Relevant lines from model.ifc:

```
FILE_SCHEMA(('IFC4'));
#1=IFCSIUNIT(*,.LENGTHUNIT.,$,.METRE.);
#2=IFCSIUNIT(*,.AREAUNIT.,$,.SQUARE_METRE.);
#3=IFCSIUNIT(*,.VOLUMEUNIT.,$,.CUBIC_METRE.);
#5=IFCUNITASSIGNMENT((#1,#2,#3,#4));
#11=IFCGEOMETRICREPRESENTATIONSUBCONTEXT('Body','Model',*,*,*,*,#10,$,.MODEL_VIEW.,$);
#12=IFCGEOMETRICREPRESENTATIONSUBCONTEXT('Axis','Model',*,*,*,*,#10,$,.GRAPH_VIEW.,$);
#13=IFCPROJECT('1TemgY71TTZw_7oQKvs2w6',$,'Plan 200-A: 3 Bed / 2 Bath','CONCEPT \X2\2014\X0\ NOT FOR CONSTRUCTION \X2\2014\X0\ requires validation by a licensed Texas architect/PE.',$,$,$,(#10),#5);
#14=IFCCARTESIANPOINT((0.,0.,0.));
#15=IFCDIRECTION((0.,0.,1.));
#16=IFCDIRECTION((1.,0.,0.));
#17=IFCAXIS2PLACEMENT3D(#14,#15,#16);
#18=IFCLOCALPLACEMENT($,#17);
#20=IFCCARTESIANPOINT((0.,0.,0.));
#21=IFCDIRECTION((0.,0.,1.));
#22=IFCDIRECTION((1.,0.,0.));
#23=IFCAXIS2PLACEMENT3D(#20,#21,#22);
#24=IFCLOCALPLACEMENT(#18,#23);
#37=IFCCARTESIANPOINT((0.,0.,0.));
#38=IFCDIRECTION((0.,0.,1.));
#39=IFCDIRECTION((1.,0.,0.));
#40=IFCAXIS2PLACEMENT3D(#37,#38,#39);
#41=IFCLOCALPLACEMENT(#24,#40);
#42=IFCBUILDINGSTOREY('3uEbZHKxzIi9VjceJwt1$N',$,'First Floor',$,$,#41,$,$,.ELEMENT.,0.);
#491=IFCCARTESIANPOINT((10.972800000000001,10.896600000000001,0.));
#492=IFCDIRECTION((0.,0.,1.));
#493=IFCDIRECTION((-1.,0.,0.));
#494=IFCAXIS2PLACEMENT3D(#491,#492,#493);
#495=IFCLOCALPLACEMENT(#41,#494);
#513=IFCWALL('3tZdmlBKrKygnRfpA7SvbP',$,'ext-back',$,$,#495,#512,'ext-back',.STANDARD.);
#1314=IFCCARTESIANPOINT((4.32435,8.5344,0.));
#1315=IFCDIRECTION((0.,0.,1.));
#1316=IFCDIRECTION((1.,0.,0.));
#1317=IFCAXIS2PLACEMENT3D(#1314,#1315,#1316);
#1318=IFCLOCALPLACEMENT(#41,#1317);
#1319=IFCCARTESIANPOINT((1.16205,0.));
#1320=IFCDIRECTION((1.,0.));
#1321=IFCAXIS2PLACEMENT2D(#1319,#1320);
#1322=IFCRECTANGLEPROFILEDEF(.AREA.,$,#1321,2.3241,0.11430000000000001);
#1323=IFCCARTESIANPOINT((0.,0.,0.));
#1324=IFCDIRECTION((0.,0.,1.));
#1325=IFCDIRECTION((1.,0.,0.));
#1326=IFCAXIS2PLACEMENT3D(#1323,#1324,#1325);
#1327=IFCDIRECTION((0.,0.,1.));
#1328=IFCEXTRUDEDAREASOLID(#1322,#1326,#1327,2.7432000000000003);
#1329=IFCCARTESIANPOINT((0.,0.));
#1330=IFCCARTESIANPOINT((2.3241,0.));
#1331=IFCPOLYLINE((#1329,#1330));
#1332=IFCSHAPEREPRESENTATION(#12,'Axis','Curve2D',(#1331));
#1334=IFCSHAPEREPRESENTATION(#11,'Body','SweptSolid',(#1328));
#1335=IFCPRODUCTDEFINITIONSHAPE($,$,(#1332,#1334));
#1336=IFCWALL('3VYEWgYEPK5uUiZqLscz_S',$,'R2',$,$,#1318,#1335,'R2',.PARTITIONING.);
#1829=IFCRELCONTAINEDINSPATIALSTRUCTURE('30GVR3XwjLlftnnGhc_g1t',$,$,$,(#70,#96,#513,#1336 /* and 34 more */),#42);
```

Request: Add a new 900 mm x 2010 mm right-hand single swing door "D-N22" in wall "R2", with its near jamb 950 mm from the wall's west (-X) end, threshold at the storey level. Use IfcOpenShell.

```python
import numpy as np
import ifcopenshell
import ifcopenshell.api.feature
import ifcopenshell.api.geometry
import ifcopenshell.api.root
import ifcopenshell.api.spatial
import ifcopenshell.geom
import ifcopenshell.util.element
import ifcopenshell.util.placement
import ifcopenshell.util.representation
import ifcopenshell.util.shape
import ifcopenshell.util.unit

model = ifcopenshell.open("model.ifc")
unit_scale = ifcopenshell.util.unit.calculate_unit_scale(model)
settings = ifcopenshell.geom.settings()


def volume(element):
    """Net volume in cubic metres, openings subtracted."""
    shape = ifcopenshell.geom.create_shape(settings, element)
    return ifcopenshell.util.shape.get_volume(shape.geometry)


wall = model.by_guid("3VYEWgYEPK5uUiZqLscz_S")
storey = ifcopenshell.util.element.get_container(wall, ifc_class="IfcBuildingStorey")
context = ifcopenshell.util.representation.get_context(model, "Model", "Body", "MODEL_VIEW")
before = volume(wall)

width, height, from_end, sill = 0.9, 2.01, 0.95, 0.0  # metres

# The wall runs along its own X axis, and the end named is its -X end.
wall_shape = ifcopenshell.geom.create_shape(settings, wall)
x, y, z = ifcopenshell.util.shape.get_vertices(wall_shape.geometry).T
start = x.min() + from_end
face, thickness = float(y.min()), float(y.max() - y.min())
wall_matrix = ifcopenshell.util.placement.get_local_placement(wall.ObjectPlacement)
level = ifcopenshell.util.placement.get_local_placement(storey.ObjectPlacement)[2, 3]


def in_wall(x, y):
    """Placement at x, y metres in the wall's axes, at sill height."""
    matrix = wall_matrix.copy()
    matrix[:, 3] = wall_matrix @ np.array([x / unit_scale, y / unit_scale, 0.0, 1.0])
    matrix[2, 3] = level + sill / unit_scale
    return matrix


# Opening: a box that overshoots both wall faces by 50 mm.
opening = ifcopenshell.api.root.create_entity(model, ifc_class="IfcOpeningElement", predefined_type="OPENING")
box = ifcopenshell.api.geometry.add_wall_representation(
    model, context=context, length=width, height=height, thickness=thickness + 0.1
)
ifcopenshell.api.geometry.assign_representation(model, product=opening, representation=box)
ifcopenshell.api.geometry.edit_object_placement(model, product=opening, matrix=in_wall(start, face - 0.05), is_si=False)
ifcopenshell.api.feature.add_feature(model, feature=opening, element=wall)

door = ifcopenshell.api.root.create_entity(model, ifc_class="IfcDoor", name="D-N22", predefined_type="DOOR")
door.OverallWidth, door.OverallHeight = width / unit_scale, height / unit_scale
door.OperationType = "SINGLE_SWING_RIGHT"
body = ifcopenshell.api.geometry.add_door_representation(
    model,
    context=context,
    overall_width=door.OverallWidth,
    overall_height=door.OverallHeight,
    operation_type="SINGLE_SWING_RIGHT",
    lining_properties={"LiningDepth": thickness / unit_scale, "ThresholdDepth": thickness / unit_scale},
)
ifcopenshell.api.geometry.assign_representation(model, product=door, representation=body)
ifcopenshell.api.spatial.assign_container(model, products=[door], relating_structure=storey)
ifcopenshell.api.feature.add_filling(model, opening=opening, element=door)

# The lining spans the wall, so the door starts at the wall face.
ifcopenshell.api.geometry.edit_object_placement(model, product=door, matrix=in_wall(start, face), is_si=False)

after = volume(wall)

print(f"wall volume {before:.3f} -> {after:.3f} m3")

model.write("model_edited.ifc")
```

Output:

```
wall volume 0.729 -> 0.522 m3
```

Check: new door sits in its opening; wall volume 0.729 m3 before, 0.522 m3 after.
